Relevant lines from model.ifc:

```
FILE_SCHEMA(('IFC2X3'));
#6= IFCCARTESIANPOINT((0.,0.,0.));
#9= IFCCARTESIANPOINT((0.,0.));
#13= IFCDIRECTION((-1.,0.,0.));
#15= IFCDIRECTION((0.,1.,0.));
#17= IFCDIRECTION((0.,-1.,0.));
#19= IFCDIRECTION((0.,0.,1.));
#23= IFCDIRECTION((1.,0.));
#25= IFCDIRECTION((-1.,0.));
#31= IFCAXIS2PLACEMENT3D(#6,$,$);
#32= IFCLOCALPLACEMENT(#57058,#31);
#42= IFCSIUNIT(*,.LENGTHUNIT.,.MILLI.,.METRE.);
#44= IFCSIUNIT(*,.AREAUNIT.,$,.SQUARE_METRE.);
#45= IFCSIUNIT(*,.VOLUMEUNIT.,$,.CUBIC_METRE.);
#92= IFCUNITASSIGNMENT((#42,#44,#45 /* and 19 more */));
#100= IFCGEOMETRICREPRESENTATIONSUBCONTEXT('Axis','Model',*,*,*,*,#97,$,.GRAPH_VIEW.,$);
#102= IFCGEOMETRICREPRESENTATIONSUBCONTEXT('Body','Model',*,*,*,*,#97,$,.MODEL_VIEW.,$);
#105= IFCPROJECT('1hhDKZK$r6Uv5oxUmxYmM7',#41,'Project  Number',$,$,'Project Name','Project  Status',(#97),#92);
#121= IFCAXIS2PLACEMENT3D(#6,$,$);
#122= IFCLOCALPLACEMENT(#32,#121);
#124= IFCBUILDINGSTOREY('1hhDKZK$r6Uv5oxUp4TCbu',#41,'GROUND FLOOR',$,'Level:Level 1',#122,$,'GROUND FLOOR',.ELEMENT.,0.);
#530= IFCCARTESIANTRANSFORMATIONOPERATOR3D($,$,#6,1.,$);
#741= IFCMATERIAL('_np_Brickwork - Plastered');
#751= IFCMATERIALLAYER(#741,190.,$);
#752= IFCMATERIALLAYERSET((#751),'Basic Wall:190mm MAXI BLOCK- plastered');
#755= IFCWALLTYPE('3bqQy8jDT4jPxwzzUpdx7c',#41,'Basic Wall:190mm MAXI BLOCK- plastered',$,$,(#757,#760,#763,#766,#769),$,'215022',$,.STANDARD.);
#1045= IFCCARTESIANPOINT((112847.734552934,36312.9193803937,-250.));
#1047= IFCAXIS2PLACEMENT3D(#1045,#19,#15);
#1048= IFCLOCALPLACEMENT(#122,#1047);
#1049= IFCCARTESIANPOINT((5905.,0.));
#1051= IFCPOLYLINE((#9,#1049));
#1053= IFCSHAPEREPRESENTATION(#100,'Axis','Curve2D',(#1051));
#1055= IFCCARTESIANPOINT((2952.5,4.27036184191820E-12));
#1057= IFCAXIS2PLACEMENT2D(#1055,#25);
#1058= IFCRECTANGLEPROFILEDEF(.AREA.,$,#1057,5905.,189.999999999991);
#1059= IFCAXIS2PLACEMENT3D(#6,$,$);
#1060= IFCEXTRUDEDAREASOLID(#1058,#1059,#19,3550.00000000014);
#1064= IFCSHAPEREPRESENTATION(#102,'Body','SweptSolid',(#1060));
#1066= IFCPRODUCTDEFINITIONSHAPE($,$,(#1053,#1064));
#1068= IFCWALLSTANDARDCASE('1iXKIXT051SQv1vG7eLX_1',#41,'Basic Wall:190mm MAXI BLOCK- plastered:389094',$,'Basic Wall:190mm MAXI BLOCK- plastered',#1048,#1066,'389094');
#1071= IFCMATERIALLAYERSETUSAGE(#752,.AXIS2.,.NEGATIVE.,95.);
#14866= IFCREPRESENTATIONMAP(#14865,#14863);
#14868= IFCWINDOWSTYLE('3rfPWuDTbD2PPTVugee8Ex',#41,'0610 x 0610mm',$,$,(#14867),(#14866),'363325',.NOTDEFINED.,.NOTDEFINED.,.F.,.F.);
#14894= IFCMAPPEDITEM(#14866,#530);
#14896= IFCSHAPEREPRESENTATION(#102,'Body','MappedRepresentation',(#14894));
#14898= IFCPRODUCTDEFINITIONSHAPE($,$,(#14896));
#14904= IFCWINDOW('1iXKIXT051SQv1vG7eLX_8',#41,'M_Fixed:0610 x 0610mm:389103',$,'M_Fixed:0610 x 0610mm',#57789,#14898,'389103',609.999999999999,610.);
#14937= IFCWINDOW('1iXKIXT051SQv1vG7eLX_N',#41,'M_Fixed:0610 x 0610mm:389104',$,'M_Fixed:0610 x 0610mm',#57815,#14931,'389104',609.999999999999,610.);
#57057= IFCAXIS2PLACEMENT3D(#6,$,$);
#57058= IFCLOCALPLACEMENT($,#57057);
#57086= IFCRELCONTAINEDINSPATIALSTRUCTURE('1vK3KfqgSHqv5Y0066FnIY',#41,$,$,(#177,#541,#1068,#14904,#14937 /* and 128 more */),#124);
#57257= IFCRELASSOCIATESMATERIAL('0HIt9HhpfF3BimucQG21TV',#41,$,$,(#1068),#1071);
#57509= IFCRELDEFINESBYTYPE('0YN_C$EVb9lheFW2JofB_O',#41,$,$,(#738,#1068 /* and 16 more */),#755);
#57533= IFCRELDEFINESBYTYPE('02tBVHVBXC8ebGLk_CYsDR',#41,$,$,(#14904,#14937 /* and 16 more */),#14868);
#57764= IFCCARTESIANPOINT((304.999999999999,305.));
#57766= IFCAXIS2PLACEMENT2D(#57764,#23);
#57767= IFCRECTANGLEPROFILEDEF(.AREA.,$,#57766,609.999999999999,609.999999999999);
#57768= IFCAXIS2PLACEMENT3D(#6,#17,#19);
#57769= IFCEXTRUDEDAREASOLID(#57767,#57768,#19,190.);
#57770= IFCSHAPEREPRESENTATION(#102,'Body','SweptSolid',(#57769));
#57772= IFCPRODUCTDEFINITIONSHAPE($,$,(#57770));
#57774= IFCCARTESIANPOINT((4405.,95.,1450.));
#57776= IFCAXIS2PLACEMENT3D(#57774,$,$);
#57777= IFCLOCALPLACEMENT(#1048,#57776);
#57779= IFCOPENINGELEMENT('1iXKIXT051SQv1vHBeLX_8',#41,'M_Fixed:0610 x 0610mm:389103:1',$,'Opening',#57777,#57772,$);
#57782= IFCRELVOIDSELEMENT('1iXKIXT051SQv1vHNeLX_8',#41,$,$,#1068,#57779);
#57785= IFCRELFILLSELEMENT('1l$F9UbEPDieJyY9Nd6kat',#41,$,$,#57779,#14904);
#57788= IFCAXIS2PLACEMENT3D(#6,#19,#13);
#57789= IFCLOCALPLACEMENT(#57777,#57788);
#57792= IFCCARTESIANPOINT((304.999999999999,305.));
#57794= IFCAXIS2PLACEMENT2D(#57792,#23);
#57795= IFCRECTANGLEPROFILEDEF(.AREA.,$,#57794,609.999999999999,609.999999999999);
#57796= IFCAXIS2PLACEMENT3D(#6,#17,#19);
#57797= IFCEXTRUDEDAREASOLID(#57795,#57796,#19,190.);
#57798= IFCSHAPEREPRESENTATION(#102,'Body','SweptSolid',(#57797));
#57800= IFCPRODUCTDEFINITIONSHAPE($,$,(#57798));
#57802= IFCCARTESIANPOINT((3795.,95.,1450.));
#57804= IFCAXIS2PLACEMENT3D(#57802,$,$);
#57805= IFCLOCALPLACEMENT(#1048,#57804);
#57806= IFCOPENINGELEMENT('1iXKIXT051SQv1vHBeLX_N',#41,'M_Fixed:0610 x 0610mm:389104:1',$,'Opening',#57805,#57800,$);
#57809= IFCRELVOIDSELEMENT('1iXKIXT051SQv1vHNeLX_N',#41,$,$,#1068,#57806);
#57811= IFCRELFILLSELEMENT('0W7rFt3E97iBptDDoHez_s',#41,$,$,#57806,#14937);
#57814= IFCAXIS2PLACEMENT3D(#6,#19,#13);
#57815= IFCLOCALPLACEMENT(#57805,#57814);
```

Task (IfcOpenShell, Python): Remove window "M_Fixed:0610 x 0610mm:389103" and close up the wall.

```python
import ifcopenshell
import ifcopenshell.api.feature
import ifcopenshell.api.root
import ifcopenshell.geom
import ifcopenshell.util.shape

model = ifcopenshell.open("model.ifc")
settings = ifcopenshell.geom.settings()


def volume(element):
    """Net volume in cubic metres, openings subtracted."""
    shape = ifcopenshell.geom.create_shape(settings, element)
    return ifcopenshell.util.shape.get_volume(shape.geometry)


window = model.by_guid("1iXKIXT051SQv1vG7eLX_8")
opening = window.FillsVoids[0].RelatingOpeningElement
wall = opening.VoidsElements[0].RelatingBuildingElement
before = volume(wall)

ifcopenshell.api.root.remove_product(model, product=window)
ifcopenshell.api.feature.remove_feature(model, feature=opening)

after = volume(wall)

print(f"wall volume {before:.3f} -> {after:.3f} m3")

model.write("model_rev.ifc")
```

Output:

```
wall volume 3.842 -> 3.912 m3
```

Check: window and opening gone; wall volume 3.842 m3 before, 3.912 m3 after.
